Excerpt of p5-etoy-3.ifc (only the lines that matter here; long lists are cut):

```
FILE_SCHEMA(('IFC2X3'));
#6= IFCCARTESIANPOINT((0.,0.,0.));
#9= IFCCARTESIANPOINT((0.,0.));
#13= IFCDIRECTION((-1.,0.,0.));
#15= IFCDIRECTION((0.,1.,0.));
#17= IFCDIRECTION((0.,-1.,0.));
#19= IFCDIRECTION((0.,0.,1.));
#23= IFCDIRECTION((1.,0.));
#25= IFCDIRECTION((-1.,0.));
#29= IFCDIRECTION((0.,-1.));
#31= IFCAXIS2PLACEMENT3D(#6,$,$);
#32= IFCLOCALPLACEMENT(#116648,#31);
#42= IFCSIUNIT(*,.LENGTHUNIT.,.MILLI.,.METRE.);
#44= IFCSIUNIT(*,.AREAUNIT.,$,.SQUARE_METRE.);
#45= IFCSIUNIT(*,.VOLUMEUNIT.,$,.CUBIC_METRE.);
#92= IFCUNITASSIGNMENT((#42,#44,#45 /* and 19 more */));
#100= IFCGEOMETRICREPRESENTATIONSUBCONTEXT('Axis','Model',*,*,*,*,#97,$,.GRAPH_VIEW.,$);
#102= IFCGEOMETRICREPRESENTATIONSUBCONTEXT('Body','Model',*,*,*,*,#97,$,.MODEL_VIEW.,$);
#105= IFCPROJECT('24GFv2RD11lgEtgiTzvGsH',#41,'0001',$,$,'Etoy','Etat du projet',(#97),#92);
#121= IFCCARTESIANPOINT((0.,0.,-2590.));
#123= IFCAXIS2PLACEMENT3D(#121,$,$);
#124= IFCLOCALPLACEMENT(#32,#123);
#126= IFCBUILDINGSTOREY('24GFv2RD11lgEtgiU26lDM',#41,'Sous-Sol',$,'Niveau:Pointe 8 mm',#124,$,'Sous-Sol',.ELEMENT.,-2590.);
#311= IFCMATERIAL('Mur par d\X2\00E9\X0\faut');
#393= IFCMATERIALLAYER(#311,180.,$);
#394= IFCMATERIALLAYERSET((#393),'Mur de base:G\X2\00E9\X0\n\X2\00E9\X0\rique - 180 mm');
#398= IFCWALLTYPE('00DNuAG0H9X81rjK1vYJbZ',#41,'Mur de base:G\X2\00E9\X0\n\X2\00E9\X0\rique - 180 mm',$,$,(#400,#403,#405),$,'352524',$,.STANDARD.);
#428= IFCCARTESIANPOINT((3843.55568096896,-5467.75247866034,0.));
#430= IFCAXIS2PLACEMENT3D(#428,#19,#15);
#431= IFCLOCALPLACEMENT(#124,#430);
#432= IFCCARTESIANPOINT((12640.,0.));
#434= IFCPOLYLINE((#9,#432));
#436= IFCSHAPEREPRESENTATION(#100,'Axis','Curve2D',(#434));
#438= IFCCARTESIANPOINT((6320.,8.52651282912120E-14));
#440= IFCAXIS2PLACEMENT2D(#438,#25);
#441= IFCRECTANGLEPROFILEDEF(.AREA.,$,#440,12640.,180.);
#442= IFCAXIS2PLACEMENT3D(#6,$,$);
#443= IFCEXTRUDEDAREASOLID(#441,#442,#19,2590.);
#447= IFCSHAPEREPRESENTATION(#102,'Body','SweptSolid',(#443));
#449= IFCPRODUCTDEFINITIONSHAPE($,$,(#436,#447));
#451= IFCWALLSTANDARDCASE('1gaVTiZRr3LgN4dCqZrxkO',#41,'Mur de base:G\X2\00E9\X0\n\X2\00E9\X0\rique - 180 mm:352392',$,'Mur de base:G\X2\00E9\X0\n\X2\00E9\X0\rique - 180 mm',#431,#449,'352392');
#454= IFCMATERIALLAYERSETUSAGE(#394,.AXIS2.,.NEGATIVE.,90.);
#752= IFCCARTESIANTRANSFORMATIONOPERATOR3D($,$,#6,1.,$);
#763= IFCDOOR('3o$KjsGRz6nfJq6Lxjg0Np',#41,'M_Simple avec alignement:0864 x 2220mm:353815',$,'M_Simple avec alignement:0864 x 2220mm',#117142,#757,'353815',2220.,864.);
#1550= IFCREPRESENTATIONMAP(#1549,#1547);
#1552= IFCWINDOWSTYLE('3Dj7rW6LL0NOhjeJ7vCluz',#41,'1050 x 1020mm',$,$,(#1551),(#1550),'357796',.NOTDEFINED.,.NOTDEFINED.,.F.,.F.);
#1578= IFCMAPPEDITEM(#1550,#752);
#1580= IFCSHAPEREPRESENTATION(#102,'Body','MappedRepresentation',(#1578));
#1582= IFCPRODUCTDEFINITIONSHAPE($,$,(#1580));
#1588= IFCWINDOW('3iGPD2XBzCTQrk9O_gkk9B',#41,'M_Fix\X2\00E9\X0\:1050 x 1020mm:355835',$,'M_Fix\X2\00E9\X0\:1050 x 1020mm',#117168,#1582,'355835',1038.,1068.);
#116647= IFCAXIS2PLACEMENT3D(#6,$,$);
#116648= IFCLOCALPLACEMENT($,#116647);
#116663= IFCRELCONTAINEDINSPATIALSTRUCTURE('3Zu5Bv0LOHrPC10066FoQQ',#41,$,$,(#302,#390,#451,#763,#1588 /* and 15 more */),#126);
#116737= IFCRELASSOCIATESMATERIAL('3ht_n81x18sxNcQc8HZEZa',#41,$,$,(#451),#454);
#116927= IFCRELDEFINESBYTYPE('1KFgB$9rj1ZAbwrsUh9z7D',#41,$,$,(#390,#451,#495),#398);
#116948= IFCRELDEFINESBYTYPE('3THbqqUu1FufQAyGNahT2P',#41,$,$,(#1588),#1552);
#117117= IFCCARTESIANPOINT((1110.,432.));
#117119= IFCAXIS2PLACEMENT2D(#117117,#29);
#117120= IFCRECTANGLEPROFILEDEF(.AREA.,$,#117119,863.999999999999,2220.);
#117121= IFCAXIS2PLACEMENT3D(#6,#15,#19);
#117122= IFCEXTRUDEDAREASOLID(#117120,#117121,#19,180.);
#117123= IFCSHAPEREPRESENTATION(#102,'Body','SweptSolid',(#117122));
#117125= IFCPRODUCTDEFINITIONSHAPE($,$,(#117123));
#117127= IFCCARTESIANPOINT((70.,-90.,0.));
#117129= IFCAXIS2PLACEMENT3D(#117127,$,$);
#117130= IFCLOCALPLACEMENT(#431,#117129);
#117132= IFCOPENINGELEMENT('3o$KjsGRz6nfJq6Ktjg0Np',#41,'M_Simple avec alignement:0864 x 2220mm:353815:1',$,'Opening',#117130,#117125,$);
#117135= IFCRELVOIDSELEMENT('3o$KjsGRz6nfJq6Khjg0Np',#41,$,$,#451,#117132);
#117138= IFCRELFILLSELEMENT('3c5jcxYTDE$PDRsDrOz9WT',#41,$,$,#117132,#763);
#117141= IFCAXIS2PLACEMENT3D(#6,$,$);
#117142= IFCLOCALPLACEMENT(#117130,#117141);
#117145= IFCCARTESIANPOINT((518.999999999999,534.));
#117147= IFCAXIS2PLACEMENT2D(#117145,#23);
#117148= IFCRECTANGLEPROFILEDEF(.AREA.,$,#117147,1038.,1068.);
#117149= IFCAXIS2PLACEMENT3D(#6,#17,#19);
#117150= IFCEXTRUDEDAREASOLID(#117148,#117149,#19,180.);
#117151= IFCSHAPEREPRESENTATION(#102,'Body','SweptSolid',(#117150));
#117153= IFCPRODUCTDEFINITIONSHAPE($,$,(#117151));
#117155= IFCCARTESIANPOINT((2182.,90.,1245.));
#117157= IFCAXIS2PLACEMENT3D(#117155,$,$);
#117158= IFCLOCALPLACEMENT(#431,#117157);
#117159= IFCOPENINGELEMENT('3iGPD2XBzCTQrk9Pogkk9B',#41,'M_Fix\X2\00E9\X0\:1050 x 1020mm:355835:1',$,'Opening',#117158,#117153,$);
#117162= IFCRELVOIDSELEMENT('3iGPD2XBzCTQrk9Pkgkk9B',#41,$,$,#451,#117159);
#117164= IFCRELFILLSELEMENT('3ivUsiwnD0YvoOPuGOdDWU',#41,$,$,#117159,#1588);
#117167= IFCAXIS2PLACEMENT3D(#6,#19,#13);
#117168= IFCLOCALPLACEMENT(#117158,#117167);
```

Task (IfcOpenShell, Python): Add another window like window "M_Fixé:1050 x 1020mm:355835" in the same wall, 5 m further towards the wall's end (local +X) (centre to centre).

```python
import ifcopenshell
import ifcopenshell.api.feature
import ifcopenshell.api.geometry
import ifcopenshell.api.root
import ifcopenshell.geom
import ifcopenshell.util.element
import ifcopenshell.util.placement
import ifcopenshell.util.shape

model = ifcopenshell.open("p5-etoy-3.ifc")
settings = ifcopenshell.geom.settings()


def volume(element):
    """Net volume in cubic metres, openings subtracted."""
    shape = ifcopenshell.geom.create_shape(settings, element)
    return ifcopenshell.util.shape.get_volume(shape.geometry)


def reuse_history(source, copy):
    """copy_class also copies each property set's owner history, people and application; keep the originals."""
    for rel in copy.IsDefinedBy:
        if rel.is_a("IfcRelDefinesByProperties") and (history := rel.RelatingPropertyDefinition.OwnerHistory):
            rel.RelatingPropertyDefinition.OwnerHistory = source.OwnerHistory
            ifcopenshell.util.element.remove_deep2(model, history)


window = model.by_id(1588)
opening = window.FillsVoids[0].RelatingOpeningElement
wall = opening.VoidsElements[0].RelatingBuildingElement
before = volume(wall)
shift = ifcopenshell.util.placement.get_local_placement(wall.ObjectPlacement)[:3, 0] * 5000.0

# copy_class copies the void relationship, type, container and properties, but no geometry.
new_opening = ifcopenshell.api.root.copy_class(model, product=opening)
new_opening.Representation = ifcopenshell.util.element.copy_deep(
    model, opening.Representation, exclude=["IfcGeometricRepresentationContext", "IfcRepresentationMap"]
)
new_opening.Name = "M_Fixé:1050 x 1020mm"
new_window = ifcopenshell.api.root.copy_class(model, product=window)
new_window.Representation = ifcopenshell.util.element.copy_deep(
    model, window.Representation, exclude=["IfcGeometricRepresentationContext", "IfcRepresentationMap"]
)
new_window.Name = "M_Fixé:1050 x 1020mm"
new_window.Tag = None
reuse_history(window, new_window)
fills = ifcopenshell.api.feature.add_filling(model, opening=new_opening, element=new_window)
fills.OwnerHistory = new_window.OwnerHistory  # required in IFC2X3

for old, new in ((opening, new_opening), (window, new_window)):
    matrix = ifcopenshell.util.placement.get_local_placement(old.ObjectPlacement)
    matrix[:3, 3] += shift
    ifcopenshell.api.geometry.edit_object_placement(model, product=new, matrix=matrix, is_si=False)

after = volume(wall)

print(f"wall volume {before:.3f} -> {after:.3f} m3")

model.write("p5-etoy-3-out.ifc")
```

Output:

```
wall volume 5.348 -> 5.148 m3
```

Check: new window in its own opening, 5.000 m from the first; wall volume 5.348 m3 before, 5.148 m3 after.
